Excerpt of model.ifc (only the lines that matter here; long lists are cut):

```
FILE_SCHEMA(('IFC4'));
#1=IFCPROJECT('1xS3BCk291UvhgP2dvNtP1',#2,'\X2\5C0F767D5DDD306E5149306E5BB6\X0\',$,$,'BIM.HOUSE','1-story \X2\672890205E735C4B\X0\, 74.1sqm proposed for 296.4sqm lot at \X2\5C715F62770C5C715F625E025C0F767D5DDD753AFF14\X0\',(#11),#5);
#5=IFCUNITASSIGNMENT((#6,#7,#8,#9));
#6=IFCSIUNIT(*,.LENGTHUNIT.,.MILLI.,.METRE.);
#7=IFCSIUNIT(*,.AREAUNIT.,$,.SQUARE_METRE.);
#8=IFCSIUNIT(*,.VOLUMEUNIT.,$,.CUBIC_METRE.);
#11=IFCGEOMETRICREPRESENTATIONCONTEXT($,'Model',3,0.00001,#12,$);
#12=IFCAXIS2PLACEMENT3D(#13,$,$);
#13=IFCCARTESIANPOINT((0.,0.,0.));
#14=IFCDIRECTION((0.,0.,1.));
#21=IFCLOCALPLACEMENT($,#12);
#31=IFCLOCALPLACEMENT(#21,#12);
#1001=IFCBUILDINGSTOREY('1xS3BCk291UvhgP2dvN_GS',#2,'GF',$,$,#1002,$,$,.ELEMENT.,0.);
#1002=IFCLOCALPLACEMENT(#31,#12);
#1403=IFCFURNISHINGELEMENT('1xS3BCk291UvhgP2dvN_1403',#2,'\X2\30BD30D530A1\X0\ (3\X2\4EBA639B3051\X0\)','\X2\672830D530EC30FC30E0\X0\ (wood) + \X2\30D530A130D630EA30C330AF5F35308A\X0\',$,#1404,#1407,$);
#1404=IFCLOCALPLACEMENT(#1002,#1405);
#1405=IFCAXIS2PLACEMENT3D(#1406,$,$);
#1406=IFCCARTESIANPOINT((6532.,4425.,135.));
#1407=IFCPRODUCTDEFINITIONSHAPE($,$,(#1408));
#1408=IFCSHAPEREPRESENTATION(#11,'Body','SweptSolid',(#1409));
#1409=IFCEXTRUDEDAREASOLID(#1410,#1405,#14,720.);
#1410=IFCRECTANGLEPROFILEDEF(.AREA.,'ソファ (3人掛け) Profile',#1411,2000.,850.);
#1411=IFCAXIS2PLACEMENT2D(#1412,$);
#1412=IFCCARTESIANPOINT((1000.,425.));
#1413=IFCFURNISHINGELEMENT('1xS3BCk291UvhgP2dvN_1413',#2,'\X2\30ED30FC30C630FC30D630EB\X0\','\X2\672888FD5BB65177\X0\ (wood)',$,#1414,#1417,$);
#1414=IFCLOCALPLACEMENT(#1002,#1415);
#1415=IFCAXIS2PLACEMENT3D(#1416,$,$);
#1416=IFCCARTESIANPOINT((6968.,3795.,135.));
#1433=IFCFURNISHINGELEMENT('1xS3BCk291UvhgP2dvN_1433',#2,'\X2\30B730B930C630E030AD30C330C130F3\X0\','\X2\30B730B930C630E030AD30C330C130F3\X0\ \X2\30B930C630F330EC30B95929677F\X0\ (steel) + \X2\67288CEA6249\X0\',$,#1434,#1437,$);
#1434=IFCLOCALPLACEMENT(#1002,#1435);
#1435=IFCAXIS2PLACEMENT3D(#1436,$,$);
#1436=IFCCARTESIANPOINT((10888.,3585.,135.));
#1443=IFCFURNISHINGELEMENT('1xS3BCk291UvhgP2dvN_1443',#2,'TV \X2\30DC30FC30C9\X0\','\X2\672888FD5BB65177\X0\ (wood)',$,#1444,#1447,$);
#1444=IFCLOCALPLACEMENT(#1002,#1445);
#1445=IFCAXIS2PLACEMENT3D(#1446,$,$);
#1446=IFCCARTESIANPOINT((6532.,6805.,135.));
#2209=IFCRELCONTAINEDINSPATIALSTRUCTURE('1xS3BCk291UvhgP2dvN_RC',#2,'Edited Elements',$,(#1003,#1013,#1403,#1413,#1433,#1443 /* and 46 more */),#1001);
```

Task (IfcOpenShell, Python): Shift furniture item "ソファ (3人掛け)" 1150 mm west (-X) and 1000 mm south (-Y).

```python
import ifcopenshell
import ifcopenshell.api.geometry
import ifcopenshell.util.placement
import ifcopenshell.util.unit

model = ifcopenshell.open("model.ifc")
unit_scale = ifcopenshell.util.unit.calculate_unit_scale(model)

item = model.by_guid("1xS3BCk291UvhgP2dvN_1403")
matrix = ifcopenshell.util.placement.get_local_placement(item.ObjectPlacement)
matrix[0, 3] -= 1.15 / unit_scale
matrix[1, 3] -= 1 / unit_scale
ifcopenshell.api.geometry.edit_object_placement(model, product=item, matrix=matrix, is_si=False)

print(ifcopenshell.util.placement.get_local_placement(item.ObjectPlacement).round(3) + 0.0)

model.write("model-out.ifc")
```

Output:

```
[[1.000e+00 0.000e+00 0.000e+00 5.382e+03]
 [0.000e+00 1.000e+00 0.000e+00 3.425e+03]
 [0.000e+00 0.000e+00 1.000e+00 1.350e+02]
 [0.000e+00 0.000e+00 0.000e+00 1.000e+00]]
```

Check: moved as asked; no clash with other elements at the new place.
